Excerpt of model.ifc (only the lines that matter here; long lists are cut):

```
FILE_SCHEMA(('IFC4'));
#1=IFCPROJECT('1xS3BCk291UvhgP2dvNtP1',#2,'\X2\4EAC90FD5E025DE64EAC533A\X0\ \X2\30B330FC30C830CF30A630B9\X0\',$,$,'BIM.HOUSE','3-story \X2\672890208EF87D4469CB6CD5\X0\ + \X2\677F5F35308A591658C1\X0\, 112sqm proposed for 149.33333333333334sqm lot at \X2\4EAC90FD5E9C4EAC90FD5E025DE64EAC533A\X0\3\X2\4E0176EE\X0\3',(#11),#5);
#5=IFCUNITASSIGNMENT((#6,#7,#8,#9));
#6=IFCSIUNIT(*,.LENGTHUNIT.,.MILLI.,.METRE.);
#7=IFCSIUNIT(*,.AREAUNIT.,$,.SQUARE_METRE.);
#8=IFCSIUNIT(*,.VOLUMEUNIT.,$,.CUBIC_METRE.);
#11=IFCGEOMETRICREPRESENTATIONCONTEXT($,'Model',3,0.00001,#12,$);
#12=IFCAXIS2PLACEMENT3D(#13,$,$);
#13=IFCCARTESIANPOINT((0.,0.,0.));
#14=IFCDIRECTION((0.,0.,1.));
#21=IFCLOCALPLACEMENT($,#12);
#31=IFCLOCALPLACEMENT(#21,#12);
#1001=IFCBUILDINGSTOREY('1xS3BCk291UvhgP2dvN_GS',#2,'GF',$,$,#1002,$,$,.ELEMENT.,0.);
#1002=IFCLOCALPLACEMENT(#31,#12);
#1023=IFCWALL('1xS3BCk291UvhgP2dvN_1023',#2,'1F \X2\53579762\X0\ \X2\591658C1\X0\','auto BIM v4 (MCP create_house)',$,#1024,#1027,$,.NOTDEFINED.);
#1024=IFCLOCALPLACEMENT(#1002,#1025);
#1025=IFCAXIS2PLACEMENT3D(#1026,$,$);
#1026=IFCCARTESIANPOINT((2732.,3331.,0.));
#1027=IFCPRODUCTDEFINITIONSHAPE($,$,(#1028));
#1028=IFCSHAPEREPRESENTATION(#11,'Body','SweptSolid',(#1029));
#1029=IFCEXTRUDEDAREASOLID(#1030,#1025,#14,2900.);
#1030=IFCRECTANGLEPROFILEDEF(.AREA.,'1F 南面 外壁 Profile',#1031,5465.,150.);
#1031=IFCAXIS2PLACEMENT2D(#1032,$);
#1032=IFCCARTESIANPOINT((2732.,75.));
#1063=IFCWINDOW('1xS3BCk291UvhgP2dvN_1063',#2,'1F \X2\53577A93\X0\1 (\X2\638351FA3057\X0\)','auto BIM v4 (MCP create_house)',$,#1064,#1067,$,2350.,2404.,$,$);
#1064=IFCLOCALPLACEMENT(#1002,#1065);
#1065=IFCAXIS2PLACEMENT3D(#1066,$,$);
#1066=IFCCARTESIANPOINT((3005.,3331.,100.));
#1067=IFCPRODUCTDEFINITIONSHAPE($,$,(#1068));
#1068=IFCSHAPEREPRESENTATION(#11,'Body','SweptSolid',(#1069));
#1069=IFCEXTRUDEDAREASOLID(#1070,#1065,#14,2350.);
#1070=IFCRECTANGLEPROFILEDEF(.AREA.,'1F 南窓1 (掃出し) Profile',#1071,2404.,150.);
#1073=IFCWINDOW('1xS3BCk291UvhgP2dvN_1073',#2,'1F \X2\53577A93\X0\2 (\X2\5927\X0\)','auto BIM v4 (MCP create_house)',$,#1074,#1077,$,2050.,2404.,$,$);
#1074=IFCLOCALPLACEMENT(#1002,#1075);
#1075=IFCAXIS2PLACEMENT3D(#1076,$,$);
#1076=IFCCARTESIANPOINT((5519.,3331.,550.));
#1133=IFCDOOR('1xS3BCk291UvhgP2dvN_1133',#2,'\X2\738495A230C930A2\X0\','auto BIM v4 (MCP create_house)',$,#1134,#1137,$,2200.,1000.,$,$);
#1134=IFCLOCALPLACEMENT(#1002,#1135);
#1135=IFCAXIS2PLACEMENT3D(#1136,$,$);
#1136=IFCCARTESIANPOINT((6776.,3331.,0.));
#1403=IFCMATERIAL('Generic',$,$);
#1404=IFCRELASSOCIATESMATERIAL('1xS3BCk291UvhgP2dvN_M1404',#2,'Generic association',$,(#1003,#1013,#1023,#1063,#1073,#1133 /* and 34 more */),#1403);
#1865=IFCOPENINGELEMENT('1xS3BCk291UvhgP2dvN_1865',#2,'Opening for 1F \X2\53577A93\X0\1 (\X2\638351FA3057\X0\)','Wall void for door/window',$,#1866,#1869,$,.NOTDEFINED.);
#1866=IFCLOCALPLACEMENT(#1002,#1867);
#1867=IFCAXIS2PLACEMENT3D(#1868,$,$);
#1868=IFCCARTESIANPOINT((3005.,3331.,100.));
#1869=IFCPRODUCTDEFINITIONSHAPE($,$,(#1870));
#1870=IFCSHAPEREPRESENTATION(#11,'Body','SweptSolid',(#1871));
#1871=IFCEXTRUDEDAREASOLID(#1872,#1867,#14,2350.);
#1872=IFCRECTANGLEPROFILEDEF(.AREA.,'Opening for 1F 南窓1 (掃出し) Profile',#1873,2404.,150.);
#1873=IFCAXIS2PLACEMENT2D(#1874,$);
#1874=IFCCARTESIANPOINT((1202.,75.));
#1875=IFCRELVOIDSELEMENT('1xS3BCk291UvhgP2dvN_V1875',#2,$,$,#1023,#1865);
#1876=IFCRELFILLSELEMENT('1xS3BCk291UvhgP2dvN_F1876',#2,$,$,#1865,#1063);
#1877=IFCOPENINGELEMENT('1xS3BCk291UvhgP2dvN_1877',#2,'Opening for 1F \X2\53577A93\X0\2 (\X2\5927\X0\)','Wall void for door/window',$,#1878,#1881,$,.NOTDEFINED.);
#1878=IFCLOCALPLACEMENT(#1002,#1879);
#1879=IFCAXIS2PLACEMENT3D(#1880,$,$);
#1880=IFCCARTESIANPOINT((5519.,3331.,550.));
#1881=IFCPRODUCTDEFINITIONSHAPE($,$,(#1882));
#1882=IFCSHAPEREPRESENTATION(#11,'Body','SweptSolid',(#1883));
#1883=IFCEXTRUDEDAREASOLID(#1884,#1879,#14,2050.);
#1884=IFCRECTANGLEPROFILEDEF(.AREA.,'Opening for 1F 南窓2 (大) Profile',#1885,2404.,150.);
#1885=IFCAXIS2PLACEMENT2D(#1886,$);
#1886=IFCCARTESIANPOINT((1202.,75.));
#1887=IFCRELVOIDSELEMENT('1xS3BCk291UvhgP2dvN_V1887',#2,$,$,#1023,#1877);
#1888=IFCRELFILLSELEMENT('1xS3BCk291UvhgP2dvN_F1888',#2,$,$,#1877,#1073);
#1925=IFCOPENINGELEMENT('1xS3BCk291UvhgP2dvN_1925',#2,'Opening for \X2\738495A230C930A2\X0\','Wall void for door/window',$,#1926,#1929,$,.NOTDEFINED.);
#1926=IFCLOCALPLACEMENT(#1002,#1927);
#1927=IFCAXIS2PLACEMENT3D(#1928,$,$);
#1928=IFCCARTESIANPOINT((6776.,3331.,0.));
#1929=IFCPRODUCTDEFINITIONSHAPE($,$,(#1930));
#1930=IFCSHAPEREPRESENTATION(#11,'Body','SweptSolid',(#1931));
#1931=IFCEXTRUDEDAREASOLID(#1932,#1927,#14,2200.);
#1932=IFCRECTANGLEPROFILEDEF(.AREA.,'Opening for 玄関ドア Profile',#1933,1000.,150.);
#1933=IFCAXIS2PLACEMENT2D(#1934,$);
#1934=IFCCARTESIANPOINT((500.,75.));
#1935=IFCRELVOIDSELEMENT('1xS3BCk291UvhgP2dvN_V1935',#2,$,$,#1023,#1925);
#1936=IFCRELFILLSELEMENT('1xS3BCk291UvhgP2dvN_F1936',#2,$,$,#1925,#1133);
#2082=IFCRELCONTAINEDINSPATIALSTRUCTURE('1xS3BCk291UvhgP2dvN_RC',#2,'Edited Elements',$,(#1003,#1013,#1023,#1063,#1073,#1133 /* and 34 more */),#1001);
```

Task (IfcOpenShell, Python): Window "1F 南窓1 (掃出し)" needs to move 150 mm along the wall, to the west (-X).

```python
import ifcopenshell
import ifcopenshell.api.geometry
import ifcopenshell.util.placement
import ifcopenshell.util.unit

model = ifcopenshell.open("model.ifc")
unit_scale = ifcopenshell.util.unit.calculate_unit_scale(model)

window = model.by_guid("1xS3BCk291UvhgP2dvN_1063")
opening = window.FillsVoids[0].RelatingOpeningElement
wall = opening.VoidsElements[0].RelatingBuildingElement

wall_matrix = ifcopenshell.util.placement.get_local_placement(wall.ObjectPlacement)
shift = wall_matrix[:3, 0] * -0.15 / unit_scale
before = ifcopenshell.util.placement.get_local_placement(window.ObjectPlacement)[:3, 3].copy()

# The window is not placed relative to its opening, so move both.
for product in (opening, window):
    matrix = ifcopenshell.util.placement.get_local_placement(product.ObjectPlacement)
    matrix[:3, 3] += shift
    ifcopenshell.api.geometry.edit_object_placement(model, product=product, matrix=matrix, is_si=False)

after = ifcopenshell.util.placement.get_local_placement(window.ObjectPlacement)[:3, 3]
print("window moved by", (after - before).round(3) + 0.0)

model.write("model-out.ifc")
```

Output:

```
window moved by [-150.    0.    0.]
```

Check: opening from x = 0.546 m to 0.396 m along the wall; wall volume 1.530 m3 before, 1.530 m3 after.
